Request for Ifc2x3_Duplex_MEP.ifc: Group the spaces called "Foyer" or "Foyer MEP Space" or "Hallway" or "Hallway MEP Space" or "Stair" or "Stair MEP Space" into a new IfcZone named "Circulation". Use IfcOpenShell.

First a look at what the model holds.

```python
import ifcopenshell

model = ifcopenshell.open("Ifc2x3_Duplex_MEP.ifc")
print(model.schema)
seen = {}
for space in model.by_type("IfcSpace"):
    seen[space.LongName] = seen.get(space.LongName, 0) + 1
for name, count in sorted(seen.items(), key=str):
    print(count, "x", name)
print("zones:", [z.Name for z in model.by_type("IfcZone")][:20])
```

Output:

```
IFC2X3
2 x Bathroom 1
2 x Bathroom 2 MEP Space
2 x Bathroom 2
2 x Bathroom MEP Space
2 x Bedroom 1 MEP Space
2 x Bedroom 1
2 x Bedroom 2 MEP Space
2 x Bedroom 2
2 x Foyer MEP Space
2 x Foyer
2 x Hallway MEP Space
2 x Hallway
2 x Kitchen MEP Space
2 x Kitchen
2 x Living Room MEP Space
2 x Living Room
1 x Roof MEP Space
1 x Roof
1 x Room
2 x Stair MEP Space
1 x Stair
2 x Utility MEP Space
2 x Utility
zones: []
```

```python
import ifcopenshell
import ifcopenshell.api.group
import ifcopenshell.api.root

model = ifcopenshell.open("Ifc2x3_Duplex_MEP.ifc")

names = {"Foyer", "Foyer MEP Space", "Hallway", "Hallway MEP Space", "Stair", "Stair MEP Space"}
spaces = [s for s in model.by_type("IfcSpace") if s.LongName in names]

zone = ifcopenshell.api.root.create_entity(model, ifc_class="IfcZone", name="Circulation")
ifcopenshell.api.group.assign_group(model, products=spaces, group=zone)
print(len(spaces), "spaces in", zone.Name)

model.write("Ifc2x3_Duplex_MEP_edited.ifc")
```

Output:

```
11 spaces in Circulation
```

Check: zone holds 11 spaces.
